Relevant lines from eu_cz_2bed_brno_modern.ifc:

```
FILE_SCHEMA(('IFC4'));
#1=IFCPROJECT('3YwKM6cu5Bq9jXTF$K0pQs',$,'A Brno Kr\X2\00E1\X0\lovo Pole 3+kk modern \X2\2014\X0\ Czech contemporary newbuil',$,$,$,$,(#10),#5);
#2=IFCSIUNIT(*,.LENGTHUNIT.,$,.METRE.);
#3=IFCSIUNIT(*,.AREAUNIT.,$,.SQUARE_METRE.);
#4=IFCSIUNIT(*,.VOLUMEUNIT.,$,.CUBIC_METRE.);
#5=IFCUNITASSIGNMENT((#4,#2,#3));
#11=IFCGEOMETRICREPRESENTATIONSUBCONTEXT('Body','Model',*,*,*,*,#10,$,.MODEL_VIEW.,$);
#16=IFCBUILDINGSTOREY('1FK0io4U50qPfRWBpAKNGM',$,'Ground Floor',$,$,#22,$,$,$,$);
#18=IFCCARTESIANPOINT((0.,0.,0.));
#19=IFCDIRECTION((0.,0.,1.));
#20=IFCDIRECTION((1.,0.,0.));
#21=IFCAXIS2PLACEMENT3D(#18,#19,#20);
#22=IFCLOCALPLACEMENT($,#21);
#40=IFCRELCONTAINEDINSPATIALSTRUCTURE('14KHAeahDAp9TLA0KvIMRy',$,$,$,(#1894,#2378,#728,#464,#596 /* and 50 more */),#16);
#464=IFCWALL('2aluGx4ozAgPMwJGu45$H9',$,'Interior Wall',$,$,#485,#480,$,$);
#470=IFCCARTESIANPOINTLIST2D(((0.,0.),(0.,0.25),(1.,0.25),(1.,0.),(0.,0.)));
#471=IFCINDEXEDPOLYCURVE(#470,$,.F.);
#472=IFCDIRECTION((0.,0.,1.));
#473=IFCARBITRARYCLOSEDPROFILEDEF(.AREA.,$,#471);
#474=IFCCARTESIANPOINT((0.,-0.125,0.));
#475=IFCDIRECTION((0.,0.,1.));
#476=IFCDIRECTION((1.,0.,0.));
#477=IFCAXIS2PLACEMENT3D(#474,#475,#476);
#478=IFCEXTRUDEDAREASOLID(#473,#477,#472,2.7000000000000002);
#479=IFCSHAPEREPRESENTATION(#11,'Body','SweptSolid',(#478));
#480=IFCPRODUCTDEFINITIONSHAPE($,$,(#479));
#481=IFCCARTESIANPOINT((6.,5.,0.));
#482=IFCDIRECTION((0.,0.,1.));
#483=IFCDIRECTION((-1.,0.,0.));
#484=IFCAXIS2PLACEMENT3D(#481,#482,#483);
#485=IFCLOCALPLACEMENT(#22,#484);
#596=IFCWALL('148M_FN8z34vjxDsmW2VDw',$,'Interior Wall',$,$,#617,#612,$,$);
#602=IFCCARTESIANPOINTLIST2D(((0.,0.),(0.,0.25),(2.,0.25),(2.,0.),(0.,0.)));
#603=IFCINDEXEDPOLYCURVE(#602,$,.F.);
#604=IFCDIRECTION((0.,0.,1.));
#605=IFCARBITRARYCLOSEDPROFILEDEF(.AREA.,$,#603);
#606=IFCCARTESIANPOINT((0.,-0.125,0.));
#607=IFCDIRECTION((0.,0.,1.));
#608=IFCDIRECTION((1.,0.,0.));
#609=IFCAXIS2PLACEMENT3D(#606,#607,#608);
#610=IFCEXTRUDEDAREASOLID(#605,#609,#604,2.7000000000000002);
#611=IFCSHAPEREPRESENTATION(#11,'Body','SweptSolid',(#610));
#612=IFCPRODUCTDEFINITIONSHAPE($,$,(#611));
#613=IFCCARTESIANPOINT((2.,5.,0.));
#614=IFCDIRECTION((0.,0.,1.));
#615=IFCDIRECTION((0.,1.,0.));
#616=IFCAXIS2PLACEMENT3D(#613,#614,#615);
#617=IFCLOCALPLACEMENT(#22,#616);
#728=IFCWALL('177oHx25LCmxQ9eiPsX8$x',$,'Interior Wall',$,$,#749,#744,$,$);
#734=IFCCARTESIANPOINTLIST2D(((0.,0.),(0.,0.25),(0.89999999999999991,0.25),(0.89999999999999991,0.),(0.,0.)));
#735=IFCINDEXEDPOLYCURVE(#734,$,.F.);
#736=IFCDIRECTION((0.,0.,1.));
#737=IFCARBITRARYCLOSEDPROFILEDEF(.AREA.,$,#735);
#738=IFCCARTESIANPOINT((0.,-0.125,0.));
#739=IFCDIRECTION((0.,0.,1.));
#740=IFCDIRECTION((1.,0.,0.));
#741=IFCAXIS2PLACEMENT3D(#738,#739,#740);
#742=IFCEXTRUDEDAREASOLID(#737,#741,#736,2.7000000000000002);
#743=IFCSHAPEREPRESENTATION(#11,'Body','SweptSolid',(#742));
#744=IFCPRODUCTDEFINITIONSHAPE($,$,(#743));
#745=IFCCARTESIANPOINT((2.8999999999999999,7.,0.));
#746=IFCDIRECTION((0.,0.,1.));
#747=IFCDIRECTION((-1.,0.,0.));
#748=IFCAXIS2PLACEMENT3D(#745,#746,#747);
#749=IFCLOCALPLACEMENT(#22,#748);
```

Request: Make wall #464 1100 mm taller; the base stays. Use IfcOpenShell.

```python
import ifcopenshell
import ifcopenshell.geom
import ifcopenshell.util.representation
import ifcopenshell.util.shape
import ifcopenshell.util.unit

model = ifcopenshell.open("eu_cz_2bed_brno_modern.ifc")
unit_scale = ifcopenshell.util.unit.calculate_unit_scale(model)
settings = ifcopenshell.geom.settings()


def volume(element):
    """Net volume in cubic metres, openings subtracted."""
    shape = ifcopenshell.geom.create_shape(settings, element)
    return ifcopenshell.util.shape.get_volume(shape.geometry)


wall = model.by_guid("2aluGx4ozAgPMwJGu45$H9")
before = volume(wall)

body = ifcopenshell.util.representation.get_representation(wall, "Model", "Body")
solid = body.Items[0]
old_height = solid.Depth
solid.Depth += 1.1 / unit_scale
after = volume(wall)

print(f"height {old_height:g} -> {solid.Depth:g}, volume {before:.3f} -> {after:.3f} m3")

model.write("eu_cz_2bed_brno_modern_edited.ifc")
```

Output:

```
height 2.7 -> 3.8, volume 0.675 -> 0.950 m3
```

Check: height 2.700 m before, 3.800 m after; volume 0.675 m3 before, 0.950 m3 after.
